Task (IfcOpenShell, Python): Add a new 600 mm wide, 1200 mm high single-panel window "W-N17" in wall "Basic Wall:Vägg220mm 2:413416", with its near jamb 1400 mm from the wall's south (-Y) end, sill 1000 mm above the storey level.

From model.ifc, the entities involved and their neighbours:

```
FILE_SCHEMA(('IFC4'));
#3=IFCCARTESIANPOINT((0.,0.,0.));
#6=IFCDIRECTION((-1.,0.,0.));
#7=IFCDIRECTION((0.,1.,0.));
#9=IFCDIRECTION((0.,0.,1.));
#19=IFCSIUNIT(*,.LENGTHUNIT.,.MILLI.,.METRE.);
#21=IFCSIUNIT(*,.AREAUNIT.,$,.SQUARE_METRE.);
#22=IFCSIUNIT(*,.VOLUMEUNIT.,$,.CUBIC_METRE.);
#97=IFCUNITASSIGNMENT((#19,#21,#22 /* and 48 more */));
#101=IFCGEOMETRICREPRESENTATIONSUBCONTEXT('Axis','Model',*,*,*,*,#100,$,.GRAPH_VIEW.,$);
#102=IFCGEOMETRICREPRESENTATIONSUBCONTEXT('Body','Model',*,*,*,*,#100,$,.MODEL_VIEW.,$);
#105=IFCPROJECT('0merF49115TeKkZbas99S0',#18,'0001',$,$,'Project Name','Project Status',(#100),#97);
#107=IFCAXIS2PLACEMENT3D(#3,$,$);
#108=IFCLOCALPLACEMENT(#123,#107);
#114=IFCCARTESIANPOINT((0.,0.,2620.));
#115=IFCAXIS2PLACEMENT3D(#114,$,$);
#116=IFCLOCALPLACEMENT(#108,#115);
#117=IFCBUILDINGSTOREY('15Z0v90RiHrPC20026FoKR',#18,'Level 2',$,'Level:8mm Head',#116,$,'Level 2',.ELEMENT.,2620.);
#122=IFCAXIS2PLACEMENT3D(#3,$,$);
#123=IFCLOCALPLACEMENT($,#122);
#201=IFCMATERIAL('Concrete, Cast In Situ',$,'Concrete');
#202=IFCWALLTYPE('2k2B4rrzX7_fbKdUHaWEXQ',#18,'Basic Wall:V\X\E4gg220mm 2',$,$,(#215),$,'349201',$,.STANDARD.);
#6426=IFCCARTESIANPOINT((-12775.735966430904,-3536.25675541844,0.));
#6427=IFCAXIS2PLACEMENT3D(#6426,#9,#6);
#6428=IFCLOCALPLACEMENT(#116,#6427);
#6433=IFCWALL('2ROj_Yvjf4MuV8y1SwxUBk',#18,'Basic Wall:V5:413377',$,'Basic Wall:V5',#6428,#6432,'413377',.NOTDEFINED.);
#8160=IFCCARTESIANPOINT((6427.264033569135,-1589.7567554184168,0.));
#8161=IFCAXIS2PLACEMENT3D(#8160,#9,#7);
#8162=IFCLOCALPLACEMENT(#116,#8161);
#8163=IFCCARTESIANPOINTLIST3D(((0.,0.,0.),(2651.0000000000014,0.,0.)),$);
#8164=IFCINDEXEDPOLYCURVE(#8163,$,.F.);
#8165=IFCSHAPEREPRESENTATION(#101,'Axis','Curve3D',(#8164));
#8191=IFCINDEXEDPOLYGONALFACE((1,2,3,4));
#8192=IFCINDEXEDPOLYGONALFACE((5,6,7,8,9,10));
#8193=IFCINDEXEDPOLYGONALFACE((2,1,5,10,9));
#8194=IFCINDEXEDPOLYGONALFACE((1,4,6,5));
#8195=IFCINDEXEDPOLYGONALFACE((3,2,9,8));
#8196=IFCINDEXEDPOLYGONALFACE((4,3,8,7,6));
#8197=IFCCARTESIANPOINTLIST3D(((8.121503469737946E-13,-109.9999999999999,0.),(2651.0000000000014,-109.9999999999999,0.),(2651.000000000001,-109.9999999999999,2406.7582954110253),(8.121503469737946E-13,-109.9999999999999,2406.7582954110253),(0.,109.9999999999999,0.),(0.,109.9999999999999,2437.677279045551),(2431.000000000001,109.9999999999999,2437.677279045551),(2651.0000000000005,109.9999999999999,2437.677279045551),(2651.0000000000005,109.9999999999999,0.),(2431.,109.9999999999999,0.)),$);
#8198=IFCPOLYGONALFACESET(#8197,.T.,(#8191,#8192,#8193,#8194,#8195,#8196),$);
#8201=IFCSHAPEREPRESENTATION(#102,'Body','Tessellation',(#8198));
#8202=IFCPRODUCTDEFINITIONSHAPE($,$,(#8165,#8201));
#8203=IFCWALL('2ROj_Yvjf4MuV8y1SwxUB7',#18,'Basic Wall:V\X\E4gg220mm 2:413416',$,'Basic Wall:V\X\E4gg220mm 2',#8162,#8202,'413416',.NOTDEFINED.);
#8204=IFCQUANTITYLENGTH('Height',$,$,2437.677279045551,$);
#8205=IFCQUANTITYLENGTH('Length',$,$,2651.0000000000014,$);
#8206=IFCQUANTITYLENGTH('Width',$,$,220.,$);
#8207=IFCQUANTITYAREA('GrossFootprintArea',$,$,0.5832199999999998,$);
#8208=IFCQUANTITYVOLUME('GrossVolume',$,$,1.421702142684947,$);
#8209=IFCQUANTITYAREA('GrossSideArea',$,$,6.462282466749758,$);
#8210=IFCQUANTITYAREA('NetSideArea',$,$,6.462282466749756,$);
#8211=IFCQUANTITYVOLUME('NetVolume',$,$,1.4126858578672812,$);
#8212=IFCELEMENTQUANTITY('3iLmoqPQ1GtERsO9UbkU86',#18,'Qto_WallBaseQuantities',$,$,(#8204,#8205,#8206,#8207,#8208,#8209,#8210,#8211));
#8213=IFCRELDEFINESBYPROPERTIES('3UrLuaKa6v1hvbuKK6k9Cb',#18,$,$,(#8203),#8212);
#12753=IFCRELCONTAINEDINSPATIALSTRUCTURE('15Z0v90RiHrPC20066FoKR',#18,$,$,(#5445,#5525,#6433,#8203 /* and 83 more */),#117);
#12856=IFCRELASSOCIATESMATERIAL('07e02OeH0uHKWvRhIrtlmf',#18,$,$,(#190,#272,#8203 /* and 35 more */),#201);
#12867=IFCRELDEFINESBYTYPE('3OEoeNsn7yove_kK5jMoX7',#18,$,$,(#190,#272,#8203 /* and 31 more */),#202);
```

```python
import numpy as np
import ifcopenshell
import ifcopenshell.api.feature
import ifcopenshell.api.geometry
import ifcopenshell.api.pset
import ifcopenshell.api.root
import ifcopenshell.api.spatial
import ifcopenshell.geom
import ifcopenshell.util.element
import ifcopenshell.util.placement
import ifcopenshell.util.representation
import ifcopenshell.util.shape
import ifcopenshell.util.unit

model = ifcopenshell.open("model.ifc")
unit_scale = ifcopenshell.util.unit.calculate_unit_scale(model)
area_scale = ifcopenshell.util.unit.calculate_unit_scale(model, "AREAUNIT")
volume_scale = ifcopenshell.util.unit.calculate_unit_scale(model, "VOLUMEUNIT")
settings = ifcopenshell.geom.settings()


def volume(element):
    """Net volume in cubic metres, openings subtracted."""
    shape = ifcopenshell.geom.create_shape(settings, element)
    return ifcopenshell.util.shape.get_volume(shape.geometry)


wall = model.by_guid("2ROj_Yvjf4MuV8y1SwxUB7")
storey = ifcopenshell.util.element.get_container(wall, ifc_class="IfcBuildingStorey")
context = ifcopenshell.util.representation.get_context(model, "Model", "Body", "MODEL_VIEW")
before = volume(wall)

width, height, from_end, sill = 0.6, 1.2, 1.4, 1  # metres

# The wall runs along its own X axis, and the end named is its -X end.
wall_shape = ifcopenshell.geom.create_shape(settings, wall)
x, y, z = ifcopenshell.util.shape.get_vertices(wall_shape.geometry).T
start = x.min() + from_end
face, thickness = float(y.min()), float(y.max() - y.min())
wall_matrix = ifcopenshell.util.placement.get_local_placement(wall.ObjectPlacement)
level = ifcopenshell.util.placement.get_local_placement(storey.ObjectPlacement)[2, 3]


def in_wall(x, y):
    """Placement at x, y metres in the wall's axes, at sill height."""
    matrix = wall_matrix.copy()
    matrix[:, 3] = wall_matrix @ np.array([x / unit_scale, y / unit_scale, 0.0, 1.0])
    matrix[2, 3] = level + sill / unit_scale
    return matrix


# Opening: a box that overshoots both wall faces by 50 mm.
opening = ifcopenshell.api.root.create_entity(model, ifc_class="IfcOpeningElement", predefined_type="OPENING")
box = ifcopenshell.api.geometry.add_wall_representation(
    model, context=context, length=width, height=height, thickness=thickness + 0.1
)
ifcopenshell.api.geometry.assign_representation(model, product=opening, representation=box)
ifcopenshell.api.geometry.edit_object_placement(model, product=opening, matrix=in_wall(start, face - 0.05), is_si=False)
ifcopenshell.api.feature.add_feature(model, feature=opening, element=wall)

window = ifcopenshell.api.root.create_entity(model, ifc_class="IfcWindow", name="W-N17", predefined_type="WINDOW")
window.OverallWidth, window.OverallHeight = width / unit_scale, height / unit_scale
window.PartitioningType = "SINGLE_PANEL"
body = ifcopenshell.api.geometry.add_window_representation(
    model,
    context=context,
    overall_width=window.OverallWidth,
    overall_height=window.OverallHeight,
    partition_type="SINGLE_PANEL",
)
ifcopenshell.api.geometry.assign_representation(model, product=window, representation=body)
ifcopenshell.api.spatial.assign_container(model, products=[window], relating_structure=storey)
ifcopenshell.api.feature.add_filling(model, opening=opening, element=window)

# Centre the window in the wall's thickness.
ifcopenshell.api.geometry.edit_object_placement(model, product=window, matrix=in_wall(start, face), is_si=False)
window_shape = ifcopenshell.geom.create_shape(settings, window)
depth = ifcopenshell.util.shape.get_vertices(window_shape.geometry)[:, 1]
offset = face + thickness / 2 - (depth.min() + depth.max()) / 2
ifcopenshell.api.geometry.edit_object_placement(model, product=window, matrix=in_wall(start, offset), is_si=False)

after = volume(wall)

# Update the wall's stored quantities.
qto = model.by_id(ifcopenshell.util.element.get_pset(wall, "Qto_WallBaseQuantities", should_inherit=False)["id"])
ifcopenshell.api.pset.edit_qto(model, qto=qto, properties={
    "NetSideArea": after / thickness / area_scale,
    "NetVolume": after / volume_scale,
})

print(f"wall volume {before:.3f} -> {after:.3f} m3")

model.write("model_v2.ifc")
```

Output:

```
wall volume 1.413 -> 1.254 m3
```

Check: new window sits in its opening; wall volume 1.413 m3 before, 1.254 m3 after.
